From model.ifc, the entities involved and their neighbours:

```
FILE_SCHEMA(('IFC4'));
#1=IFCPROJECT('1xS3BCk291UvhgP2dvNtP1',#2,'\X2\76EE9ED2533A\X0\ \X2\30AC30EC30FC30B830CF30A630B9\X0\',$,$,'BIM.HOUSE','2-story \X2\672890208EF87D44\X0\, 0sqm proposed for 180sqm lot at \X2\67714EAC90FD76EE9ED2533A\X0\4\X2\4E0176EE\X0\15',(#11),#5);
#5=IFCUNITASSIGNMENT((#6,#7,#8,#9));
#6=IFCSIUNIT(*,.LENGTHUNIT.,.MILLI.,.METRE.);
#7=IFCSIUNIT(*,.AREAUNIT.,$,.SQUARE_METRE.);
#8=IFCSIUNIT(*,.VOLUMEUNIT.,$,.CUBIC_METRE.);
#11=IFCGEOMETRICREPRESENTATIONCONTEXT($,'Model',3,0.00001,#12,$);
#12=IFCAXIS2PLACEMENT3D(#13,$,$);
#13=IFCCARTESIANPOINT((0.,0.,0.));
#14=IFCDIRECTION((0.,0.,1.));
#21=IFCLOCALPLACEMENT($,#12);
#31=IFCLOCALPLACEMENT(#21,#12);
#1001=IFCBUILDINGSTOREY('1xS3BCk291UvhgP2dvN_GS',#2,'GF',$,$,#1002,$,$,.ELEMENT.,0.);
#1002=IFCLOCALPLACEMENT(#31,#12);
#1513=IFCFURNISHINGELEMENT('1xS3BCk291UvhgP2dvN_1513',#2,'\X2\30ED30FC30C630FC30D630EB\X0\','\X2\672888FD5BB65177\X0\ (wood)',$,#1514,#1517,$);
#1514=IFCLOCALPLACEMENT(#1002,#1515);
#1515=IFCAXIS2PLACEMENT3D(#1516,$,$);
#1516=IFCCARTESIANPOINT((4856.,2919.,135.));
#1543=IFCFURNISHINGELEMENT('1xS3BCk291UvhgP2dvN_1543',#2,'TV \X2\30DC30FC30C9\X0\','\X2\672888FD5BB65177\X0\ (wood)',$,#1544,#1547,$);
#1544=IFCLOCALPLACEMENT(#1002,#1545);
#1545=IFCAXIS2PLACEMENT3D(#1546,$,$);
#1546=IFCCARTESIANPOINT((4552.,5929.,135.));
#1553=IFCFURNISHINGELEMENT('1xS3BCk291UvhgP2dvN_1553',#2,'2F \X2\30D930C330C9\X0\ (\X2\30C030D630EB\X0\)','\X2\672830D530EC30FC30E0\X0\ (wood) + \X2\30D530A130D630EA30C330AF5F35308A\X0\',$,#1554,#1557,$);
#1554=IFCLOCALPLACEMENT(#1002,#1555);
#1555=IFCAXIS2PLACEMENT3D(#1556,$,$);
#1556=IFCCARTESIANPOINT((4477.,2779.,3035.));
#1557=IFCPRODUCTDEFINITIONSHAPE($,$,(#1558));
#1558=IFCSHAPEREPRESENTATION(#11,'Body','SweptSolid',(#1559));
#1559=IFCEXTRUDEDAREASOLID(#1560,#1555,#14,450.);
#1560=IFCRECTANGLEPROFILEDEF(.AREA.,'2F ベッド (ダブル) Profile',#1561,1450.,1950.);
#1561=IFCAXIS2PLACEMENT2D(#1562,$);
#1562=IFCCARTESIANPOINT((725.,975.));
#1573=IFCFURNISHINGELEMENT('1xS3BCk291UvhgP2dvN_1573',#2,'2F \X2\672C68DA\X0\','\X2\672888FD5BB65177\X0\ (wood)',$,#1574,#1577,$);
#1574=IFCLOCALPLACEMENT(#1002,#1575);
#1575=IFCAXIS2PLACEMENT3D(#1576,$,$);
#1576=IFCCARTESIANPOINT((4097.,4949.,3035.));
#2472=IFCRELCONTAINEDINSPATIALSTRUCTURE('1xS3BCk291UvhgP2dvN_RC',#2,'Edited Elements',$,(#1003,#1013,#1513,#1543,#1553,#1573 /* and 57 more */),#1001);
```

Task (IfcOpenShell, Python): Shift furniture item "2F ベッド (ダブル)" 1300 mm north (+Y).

```python
import ifcopenshell
import ifcopenshell.api.geometry
import ifcopenshell.util.placement
import ifcopenshell.util.unit

model = ifcopenshell.open("model.ifc")
unit_scale = ifcopenshell.util.unit.calculate_unit_scale(model)

item = model.by_id(1553)
matrix = ifcopenshell.util.placement.get_local_placement(item.ObjectPlacement)
matrix[1, 3] += 1.3 / unit_scale
ifcopenshell.api.geometry.edit_object_placement(model, product=item, matrix=matrix, is_si=False)

print(ifcopenshell.util.placement.get_local_placement(item.ObjectPlacement).round(3) + 0.0)

model.write("model_edited.ifc")
```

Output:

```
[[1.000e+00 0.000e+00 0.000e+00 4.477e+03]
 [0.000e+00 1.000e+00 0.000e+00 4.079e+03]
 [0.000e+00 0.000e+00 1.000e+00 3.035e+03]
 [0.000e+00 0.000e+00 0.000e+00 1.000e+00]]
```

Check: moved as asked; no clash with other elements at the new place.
